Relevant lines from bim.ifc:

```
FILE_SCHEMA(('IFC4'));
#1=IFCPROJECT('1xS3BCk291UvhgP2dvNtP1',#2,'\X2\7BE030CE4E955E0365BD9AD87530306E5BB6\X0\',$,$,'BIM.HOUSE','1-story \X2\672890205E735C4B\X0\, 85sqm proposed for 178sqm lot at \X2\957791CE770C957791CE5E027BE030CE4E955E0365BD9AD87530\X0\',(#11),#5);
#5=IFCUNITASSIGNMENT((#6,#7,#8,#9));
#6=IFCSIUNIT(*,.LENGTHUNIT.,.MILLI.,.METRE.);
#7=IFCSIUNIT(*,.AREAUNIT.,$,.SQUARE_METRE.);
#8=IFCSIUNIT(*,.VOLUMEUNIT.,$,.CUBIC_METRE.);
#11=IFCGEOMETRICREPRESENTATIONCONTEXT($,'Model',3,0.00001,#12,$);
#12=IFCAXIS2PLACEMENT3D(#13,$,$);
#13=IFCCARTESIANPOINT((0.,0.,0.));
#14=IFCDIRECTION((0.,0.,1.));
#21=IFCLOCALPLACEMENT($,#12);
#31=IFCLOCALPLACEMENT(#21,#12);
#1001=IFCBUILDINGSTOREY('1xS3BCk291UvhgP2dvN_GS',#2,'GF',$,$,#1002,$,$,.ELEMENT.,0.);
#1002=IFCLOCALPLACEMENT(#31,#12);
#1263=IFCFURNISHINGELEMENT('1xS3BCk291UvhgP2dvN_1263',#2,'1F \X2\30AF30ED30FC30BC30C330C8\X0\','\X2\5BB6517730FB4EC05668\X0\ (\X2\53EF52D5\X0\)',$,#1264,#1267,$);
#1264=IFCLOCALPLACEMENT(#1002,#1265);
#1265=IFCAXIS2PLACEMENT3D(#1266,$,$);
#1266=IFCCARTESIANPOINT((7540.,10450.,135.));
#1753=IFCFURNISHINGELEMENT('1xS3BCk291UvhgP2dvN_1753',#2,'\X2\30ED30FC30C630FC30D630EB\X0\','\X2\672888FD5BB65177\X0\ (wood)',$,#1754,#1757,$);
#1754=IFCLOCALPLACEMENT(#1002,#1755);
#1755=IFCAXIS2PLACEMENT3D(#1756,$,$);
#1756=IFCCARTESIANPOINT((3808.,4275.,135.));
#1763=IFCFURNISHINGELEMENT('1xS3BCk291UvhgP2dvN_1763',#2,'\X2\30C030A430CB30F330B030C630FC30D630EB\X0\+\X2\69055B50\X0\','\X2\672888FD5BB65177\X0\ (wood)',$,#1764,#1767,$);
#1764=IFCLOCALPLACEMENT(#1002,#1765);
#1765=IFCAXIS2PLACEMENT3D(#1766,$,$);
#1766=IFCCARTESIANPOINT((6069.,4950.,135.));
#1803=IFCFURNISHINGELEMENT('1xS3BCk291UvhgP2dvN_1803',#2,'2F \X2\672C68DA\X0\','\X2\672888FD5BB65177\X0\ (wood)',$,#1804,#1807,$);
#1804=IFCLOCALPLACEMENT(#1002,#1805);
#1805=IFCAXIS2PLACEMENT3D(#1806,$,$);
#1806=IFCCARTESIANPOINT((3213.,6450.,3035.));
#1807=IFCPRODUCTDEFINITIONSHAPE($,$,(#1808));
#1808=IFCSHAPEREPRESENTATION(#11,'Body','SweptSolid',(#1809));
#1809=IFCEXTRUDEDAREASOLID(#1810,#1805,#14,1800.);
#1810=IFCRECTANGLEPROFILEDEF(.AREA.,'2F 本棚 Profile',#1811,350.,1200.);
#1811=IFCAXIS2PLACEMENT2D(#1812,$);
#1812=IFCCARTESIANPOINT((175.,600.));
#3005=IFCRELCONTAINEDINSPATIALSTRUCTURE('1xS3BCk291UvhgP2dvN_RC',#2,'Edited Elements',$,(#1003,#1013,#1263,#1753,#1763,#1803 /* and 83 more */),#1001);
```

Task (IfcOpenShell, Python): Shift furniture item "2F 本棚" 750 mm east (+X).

```python
import ifcopenshell
import ifcopenshell.api.geometry
import ifcopenshell.util.placement
import ifcopenshell.util.unit

model = ifcopenshell.open("bim.ifc")
unit_scale = ifcopenshell.util.unit.calculate_unit_scale(model)

item = model.by_id(1803)
matrix = ifcopenshell.util.placement.get_local_placement(item.ObjectPlacement)
matrix[0, 3] += 0.75 / unit_scale
ifcopenshell.api.geometry.edit_object_placement(model, product=item, matrix=matrix, is_si=False)

print(ifcopenshell.util.placement.get_local_placement(item.ObjectPlacement).round(3) + 0.0)

model.write("bim_rev.ifc")
```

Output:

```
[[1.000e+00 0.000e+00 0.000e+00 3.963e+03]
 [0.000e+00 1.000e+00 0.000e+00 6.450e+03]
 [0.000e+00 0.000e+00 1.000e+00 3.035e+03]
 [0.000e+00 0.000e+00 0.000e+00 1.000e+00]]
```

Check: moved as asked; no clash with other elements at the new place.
